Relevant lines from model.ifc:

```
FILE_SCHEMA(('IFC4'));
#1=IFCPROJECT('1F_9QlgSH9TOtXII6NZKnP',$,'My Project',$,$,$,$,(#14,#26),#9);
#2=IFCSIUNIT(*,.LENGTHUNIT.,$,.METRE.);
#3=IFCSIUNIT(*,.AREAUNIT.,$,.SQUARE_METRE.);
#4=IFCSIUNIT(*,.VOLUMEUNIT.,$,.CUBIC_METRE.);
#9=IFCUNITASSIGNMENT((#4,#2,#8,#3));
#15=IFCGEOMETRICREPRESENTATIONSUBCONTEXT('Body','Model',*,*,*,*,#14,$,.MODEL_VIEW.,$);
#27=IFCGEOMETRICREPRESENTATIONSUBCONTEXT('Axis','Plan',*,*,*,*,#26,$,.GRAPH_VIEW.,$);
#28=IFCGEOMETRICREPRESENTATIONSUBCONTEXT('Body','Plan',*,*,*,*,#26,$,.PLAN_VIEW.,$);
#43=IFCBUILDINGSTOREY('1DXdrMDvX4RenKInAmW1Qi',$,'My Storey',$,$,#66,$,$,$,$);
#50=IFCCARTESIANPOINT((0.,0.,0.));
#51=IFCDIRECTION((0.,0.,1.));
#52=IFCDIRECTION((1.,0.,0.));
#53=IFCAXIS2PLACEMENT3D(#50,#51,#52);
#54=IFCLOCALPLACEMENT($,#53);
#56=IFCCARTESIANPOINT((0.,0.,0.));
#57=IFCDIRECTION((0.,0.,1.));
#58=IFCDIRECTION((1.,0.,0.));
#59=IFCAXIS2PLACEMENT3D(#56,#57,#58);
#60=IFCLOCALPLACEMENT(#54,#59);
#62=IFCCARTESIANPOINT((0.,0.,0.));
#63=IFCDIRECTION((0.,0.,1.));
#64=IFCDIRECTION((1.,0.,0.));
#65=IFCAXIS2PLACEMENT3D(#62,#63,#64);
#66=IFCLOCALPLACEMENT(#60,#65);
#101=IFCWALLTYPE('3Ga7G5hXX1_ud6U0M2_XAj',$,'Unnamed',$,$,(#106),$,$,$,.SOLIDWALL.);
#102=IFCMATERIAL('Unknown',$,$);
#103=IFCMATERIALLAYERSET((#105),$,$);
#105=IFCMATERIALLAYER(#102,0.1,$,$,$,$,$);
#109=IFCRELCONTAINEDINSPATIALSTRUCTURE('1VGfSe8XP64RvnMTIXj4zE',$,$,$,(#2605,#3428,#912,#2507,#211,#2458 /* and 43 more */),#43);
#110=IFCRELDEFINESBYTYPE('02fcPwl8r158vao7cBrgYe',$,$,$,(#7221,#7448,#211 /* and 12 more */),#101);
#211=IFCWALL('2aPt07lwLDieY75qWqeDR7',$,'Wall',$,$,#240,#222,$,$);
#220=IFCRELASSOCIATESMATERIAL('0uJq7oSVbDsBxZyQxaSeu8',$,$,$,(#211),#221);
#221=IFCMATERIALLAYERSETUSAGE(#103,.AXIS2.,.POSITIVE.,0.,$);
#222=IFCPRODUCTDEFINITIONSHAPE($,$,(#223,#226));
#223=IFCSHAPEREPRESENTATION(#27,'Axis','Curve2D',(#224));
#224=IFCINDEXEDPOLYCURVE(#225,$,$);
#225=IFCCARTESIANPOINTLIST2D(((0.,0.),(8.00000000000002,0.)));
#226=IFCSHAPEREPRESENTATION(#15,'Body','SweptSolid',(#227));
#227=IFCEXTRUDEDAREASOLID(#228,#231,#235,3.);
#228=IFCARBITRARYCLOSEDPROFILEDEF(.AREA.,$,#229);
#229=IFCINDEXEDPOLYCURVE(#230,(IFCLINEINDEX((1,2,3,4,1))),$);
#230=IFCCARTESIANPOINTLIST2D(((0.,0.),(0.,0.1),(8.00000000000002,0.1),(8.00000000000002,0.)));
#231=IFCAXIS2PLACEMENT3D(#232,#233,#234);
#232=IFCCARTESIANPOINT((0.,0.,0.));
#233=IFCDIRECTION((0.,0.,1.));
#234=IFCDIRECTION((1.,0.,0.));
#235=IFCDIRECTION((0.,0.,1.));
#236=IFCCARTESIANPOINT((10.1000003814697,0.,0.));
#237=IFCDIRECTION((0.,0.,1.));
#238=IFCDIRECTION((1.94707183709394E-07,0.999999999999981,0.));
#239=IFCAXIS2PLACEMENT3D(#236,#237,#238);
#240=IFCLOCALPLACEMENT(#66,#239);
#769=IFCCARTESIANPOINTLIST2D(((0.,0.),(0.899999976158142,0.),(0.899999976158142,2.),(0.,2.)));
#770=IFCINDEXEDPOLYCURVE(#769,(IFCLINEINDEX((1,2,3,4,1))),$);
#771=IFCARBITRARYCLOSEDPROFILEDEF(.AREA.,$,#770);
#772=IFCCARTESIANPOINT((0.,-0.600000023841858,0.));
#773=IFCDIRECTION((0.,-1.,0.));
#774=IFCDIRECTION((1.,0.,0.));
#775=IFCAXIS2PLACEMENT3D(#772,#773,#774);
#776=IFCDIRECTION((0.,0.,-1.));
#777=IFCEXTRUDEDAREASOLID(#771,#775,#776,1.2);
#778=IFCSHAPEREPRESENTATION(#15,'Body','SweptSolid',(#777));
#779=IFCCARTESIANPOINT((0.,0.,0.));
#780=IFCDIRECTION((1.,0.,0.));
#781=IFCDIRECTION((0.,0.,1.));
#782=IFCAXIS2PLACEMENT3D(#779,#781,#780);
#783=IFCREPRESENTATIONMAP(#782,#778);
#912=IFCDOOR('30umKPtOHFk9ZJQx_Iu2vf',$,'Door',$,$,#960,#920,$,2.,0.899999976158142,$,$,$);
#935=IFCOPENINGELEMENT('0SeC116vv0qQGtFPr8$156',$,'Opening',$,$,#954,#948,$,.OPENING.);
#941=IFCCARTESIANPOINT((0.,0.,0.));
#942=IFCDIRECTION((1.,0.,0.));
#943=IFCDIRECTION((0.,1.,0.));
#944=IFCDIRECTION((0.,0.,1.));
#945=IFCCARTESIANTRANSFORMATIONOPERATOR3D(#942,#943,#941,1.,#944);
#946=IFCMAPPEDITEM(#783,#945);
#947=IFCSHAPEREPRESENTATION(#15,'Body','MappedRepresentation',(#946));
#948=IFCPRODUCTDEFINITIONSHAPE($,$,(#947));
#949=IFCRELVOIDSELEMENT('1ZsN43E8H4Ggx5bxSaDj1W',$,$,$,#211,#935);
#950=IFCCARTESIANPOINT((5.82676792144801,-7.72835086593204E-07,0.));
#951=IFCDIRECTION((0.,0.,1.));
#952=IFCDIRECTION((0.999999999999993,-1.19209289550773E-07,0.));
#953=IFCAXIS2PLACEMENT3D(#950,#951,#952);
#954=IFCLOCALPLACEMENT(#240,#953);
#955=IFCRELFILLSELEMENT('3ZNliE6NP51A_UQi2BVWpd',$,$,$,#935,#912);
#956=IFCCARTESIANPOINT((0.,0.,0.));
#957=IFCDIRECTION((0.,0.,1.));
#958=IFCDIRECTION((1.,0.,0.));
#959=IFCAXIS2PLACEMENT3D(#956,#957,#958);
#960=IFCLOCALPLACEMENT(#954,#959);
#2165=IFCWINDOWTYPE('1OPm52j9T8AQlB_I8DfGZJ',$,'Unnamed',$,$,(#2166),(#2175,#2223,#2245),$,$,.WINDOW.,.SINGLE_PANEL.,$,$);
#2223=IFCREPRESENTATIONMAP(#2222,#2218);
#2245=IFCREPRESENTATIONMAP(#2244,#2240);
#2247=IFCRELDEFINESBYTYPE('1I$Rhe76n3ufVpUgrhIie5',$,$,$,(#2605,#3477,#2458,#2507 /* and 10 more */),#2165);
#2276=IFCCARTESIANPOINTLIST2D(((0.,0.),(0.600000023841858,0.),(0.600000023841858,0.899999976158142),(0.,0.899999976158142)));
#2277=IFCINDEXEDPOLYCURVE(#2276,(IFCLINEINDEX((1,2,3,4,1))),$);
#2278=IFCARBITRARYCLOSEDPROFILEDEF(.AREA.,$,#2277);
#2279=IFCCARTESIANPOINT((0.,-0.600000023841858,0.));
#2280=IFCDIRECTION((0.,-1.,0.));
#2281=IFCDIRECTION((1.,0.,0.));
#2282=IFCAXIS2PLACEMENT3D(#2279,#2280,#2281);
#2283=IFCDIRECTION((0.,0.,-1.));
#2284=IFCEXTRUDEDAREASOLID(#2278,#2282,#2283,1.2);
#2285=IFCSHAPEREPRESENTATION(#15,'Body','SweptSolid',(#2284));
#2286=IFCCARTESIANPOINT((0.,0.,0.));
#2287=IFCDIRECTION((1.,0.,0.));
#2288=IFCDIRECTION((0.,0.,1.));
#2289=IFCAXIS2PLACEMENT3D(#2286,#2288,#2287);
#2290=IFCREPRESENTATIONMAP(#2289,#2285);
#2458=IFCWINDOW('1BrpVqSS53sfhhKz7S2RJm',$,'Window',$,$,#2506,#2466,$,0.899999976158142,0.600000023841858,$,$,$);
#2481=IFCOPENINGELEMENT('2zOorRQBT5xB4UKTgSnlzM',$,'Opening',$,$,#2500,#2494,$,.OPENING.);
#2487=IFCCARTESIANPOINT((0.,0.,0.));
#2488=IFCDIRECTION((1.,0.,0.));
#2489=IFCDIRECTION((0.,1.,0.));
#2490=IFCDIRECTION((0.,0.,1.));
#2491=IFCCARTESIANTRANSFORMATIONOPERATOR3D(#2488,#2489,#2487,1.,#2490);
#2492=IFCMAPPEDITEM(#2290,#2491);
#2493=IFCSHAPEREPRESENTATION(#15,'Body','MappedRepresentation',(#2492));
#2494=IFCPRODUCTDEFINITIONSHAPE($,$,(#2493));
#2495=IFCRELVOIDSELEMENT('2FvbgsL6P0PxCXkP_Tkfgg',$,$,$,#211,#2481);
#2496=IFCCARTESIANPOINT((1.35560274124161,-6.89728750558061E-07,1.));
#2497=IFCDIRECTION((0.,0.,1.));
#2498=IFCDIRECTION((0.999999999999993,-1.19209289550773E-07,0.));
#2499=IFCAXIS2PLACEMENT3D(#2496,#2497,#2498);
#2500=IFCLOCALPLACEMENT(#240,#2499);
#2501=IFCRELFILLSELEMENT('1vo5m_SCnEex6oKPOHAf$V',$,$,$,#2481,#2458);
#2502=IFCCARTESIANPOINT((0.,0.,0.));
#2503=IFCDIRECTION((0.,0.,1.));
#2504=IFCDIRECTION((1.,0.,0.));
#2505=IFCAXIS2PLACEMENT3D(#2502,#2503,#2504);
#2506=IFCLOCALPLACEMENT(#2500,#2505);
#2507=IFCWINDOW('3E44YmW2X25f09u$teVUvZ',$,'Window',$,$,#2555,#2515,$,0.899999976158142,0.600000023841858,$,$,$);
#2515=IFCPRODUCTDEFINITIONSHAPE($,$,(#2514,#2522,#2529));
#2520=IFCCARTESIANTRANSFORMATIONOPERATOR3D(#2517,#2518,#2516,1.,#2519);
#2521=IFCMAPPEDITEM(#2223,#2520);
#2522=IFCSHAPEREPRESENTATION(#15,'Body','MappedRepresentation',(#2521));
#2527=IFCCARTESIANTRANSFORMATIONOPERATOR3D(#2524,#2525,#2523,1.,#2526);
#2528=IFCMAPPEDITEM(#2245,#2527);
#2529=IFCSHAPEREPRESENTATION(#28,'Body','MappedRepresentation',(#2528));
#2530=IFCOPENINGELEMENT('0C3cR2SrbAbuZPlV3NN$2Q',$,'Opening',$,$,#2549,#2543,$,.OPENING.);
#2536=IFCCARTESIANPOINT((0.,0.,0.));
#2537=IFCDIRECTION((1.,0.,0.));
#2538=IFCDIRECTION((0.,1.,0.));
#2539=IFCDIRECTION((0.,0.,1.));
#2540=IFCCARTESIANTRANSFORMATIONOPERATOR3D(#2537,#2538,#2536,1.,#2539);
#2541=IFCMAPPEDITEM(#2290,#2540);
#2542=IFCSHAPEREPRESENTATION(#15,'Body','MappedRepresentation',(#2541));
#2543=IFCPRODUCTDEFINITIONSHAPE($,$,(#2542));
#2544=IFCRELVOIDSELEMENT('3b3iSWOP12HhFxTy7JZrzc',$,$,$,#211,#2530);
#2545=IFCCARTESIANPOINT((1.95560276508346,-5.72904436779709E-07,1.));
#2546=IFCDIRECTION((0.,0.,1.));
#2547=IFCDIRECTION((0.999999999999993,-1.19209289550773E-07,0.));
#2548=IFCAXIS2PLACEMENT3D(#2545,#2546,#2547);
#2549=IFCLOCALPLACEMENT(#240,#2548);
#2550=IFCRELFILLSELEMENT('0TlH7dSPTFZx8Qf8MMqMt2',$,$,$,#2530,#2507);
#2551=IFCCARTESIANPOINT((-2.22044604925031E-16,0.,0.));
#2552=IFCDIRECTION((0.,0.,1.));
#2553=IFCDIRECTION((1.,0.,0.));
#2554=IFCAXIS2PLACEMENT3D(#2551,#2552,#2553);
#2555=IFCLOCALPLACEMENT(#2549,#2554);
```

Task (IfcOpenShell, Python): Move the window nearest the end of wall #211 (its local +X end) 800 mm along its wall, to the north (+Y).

```python
import ifcopenshell
import ifcopenshell.api.geometry
import ifcopenshell.util.placement
import ifcopenshell.util.unit

model = ifcopenshell.open("model.ifc")
unit_scale = ifcopenshell.util.unit.calculate_unit_scale(model)

window = model.by_guid("3E44YmW2X25f09u$teVUvZ")
opening = window.FillsVoids[0].RelatingOpeningElement
wall = opening.VoidsElements[0].RelatingBuildingElement

wall_matrix = ifcopenshell.util.placement.get_local_placement(wall.ObjectPlacement)
shift = wall_matrix[:3, 0] * 0.8 / unit_scale
before = ifcopenshell.util.placement.get_local_placement(window.ObjectPlacement)[:3, 3].copy()

# The window is placed relative to its opening, so it follows when the opening moves.
matrix = ifcopenshell.util.placement.get_local_placement(opening.ObjectPlacement)
matrix[:3, 3] += shift
ifcopenshell.api.geometry.edit_object_placement(
    model, product=opening, matrix=matrix, is_si=False, should_transform_children=True
)

after = ifcopenshell.util.placement.get_local_placement(window.ObjectPlacement)[:3, 3]
print("window moved by", (after - before).round(3) + 0.0)

model.write("model_rev.ifc")
```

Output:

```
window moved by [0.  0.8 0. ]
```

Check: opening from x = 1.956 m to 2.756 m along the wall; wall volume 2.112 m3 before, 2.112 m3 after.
